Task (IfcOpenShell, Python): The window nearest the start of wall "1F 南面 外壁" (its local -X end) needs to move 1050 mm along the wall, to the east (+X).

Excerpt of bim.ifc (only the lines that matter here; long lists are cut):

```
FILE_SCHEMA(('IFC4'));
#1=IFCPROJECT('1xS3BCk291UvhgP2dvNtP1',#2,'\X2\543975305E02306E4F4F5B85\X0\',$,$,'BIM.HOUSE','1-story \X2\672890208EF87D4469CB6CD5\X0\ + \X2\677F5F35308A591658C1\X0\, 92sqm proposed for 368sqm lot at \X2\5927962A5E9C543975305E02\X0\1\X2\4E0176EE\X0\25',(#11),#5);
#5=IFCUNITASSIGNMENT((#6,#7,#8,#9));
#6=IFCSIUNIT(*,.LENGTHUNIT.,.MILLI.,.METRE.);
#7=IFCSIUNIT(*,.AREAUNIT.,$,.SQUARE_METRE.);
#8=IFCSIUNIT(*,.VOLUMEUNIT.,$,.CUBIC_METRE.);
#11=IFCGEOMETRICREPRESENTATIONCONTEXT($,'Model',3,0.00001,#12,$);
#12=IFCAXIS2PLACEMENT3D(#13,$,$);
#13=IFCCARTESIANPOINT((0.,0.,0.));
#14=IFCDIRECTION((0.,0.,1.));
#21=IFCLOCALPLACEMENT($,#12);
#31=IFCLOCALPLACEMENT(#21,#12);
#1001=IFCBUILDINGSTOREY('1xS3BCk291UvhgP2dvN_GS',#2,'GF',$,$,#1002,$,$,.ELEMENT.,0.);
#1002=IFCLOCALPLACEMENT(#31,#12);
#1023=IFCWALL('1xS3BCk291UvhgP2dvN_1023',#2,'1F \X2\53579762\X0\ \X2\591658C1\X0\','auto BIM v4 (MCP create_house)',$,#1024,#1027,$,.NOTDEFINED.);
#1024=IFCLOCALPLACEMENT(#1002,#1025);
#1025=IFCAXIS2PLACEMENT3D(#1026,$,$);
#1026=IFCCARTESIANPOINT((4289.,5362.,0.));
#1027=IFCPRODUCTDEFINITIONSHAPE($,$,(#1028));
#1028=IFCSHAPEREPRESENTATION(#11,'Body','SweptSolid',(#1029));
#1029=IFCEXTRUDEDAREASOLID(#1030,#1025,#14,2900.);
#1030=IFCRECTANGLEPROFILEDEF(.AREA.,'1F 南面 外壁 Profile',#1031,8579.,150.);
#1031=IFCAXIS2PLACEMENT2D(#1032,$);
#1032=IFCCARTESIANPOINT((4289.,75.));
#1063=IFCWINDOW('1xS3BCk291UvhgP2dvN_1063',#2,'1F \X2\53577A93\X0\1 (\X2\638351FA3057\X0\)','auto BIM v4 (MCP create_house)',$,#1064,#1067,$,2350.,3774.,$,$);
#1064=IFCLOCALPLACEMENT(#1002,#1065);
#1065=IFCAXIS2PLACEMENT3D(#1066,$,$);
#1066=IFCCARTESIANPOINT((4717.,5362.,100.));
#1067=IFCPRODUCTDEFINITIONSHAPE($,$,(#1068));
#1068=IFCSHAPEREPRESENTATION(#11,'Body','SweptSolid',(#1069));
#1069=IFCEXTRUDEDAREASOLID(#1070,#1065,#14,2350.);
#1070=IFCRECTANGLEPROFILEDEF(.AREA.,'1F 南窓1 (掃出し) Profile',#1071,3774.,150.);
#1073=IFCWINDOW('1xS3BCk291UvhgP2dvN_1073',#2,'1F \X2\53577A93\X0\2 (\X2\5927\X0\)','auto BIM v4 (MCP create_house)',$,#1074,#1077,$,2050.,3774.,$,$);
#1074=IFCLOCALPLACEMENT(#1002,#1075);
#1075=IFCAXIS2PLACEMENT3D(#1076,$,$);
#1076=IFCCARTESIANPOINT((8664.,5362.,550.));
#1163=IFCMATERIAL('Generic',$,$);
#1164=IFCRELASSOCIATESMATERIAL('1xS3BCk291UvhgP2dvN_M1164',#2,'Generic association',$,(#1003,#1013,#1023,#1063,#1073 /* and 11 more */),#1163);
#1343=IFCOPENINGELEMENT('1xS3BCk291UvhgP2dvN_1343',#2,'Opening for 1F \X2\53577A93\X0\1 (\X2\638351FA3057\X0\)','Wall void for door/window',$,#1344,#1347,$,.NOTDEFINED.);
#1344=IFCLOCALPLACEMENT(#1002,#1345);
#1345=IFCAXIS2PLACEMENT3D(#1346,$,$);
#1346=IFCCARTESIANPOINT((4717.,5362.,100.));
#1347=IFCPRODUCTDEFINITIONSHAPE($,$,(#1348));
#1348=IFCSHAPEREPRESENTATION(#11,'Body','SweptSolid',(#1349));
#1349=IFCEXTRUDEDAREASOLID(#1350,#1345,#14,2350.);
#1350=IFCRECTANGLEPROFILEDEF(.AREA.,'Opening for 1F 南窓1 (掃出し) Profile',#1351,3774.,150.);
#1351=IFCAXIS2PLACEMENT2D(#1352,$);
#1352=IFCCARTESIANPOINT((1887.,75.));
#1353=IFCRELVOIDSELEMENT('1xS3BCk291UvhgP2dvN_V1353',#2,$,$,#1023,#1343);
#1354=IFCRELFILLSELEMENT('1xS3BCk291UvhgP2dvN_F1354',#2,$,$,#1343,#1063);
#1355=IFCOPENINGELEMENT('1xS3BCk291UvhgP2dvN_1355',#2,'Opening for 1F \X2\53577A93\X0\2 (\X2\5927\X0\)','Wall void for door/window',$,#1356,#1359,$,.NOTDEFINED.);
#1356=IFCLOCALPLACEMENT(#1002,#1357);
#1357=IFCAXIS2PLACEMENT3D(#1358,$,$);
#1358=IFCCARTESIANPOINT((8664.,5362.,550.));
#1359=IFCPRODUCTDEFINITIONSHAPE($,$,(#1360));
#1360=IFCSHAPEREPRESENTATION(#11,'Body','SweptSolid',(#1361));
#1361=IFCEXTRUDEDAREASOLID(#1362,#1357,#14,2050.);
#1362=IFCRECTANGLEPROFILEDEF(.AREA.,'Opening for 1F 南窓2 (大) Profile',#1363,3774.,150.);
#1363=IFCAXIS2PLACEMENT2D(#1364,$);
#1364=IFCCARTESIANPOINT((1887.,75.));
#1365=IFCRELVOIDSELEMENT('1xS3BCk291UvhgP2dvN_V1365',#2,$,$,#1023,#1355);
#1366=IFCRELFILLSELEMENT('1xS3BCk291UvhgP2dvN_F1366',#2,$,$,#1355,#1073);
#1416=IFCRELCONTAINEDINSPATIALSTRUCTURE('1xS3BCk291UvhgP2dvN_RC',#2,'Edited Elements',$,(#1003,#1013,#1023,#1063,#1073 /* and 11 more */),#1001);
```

```python
import ifcopenshell
import ifcopenshell.api.geometry
import ifcopenshell.util.placement
import ifcopenshell.util.unit

model = ifcopenshell.open("bim.ifc")
unit_scale = ifcopenshell.util.unit.calculate_unit_scale(model)

window = model.by_id(1063)
opening = window.FillsVoids[0].RelatingOpeningElement
wall = opening.VoidsElements[0].RelatingBuildingElement

wall_matrix = ifcopenshell.util.placement.get_local_placement(wall.ObjectPlacement)
shift = wall_matrix[:3, 0] * 1.05 / unit_scale
before = ifcopenshell.util.placement.get_local_placement(window.ObjectPlacement)[:3, 3].copy()

# The window is not placed relative to its opening, so move both.
for product in (opening, window):
    matrix = ifcopenshell.util.placement.get_local_placement(product.ObjectPlacement)
    matrix[:3, 3] += shift
    ifcopenshell.api.geometry.edit_object_placement(model, product=product, matrix=matrix, is_si=False)

after = ifcopenshell.util.placement.get_local_placement(window.ObjectPlacement)[:3, 3]
print("window moved by", (after - before).round(3) + 0.0)

model.write("bim_updated.ifc")
```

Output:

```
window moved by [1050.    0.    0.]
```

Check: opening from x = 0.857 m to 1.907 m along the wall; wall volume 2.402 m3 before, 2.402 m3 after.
